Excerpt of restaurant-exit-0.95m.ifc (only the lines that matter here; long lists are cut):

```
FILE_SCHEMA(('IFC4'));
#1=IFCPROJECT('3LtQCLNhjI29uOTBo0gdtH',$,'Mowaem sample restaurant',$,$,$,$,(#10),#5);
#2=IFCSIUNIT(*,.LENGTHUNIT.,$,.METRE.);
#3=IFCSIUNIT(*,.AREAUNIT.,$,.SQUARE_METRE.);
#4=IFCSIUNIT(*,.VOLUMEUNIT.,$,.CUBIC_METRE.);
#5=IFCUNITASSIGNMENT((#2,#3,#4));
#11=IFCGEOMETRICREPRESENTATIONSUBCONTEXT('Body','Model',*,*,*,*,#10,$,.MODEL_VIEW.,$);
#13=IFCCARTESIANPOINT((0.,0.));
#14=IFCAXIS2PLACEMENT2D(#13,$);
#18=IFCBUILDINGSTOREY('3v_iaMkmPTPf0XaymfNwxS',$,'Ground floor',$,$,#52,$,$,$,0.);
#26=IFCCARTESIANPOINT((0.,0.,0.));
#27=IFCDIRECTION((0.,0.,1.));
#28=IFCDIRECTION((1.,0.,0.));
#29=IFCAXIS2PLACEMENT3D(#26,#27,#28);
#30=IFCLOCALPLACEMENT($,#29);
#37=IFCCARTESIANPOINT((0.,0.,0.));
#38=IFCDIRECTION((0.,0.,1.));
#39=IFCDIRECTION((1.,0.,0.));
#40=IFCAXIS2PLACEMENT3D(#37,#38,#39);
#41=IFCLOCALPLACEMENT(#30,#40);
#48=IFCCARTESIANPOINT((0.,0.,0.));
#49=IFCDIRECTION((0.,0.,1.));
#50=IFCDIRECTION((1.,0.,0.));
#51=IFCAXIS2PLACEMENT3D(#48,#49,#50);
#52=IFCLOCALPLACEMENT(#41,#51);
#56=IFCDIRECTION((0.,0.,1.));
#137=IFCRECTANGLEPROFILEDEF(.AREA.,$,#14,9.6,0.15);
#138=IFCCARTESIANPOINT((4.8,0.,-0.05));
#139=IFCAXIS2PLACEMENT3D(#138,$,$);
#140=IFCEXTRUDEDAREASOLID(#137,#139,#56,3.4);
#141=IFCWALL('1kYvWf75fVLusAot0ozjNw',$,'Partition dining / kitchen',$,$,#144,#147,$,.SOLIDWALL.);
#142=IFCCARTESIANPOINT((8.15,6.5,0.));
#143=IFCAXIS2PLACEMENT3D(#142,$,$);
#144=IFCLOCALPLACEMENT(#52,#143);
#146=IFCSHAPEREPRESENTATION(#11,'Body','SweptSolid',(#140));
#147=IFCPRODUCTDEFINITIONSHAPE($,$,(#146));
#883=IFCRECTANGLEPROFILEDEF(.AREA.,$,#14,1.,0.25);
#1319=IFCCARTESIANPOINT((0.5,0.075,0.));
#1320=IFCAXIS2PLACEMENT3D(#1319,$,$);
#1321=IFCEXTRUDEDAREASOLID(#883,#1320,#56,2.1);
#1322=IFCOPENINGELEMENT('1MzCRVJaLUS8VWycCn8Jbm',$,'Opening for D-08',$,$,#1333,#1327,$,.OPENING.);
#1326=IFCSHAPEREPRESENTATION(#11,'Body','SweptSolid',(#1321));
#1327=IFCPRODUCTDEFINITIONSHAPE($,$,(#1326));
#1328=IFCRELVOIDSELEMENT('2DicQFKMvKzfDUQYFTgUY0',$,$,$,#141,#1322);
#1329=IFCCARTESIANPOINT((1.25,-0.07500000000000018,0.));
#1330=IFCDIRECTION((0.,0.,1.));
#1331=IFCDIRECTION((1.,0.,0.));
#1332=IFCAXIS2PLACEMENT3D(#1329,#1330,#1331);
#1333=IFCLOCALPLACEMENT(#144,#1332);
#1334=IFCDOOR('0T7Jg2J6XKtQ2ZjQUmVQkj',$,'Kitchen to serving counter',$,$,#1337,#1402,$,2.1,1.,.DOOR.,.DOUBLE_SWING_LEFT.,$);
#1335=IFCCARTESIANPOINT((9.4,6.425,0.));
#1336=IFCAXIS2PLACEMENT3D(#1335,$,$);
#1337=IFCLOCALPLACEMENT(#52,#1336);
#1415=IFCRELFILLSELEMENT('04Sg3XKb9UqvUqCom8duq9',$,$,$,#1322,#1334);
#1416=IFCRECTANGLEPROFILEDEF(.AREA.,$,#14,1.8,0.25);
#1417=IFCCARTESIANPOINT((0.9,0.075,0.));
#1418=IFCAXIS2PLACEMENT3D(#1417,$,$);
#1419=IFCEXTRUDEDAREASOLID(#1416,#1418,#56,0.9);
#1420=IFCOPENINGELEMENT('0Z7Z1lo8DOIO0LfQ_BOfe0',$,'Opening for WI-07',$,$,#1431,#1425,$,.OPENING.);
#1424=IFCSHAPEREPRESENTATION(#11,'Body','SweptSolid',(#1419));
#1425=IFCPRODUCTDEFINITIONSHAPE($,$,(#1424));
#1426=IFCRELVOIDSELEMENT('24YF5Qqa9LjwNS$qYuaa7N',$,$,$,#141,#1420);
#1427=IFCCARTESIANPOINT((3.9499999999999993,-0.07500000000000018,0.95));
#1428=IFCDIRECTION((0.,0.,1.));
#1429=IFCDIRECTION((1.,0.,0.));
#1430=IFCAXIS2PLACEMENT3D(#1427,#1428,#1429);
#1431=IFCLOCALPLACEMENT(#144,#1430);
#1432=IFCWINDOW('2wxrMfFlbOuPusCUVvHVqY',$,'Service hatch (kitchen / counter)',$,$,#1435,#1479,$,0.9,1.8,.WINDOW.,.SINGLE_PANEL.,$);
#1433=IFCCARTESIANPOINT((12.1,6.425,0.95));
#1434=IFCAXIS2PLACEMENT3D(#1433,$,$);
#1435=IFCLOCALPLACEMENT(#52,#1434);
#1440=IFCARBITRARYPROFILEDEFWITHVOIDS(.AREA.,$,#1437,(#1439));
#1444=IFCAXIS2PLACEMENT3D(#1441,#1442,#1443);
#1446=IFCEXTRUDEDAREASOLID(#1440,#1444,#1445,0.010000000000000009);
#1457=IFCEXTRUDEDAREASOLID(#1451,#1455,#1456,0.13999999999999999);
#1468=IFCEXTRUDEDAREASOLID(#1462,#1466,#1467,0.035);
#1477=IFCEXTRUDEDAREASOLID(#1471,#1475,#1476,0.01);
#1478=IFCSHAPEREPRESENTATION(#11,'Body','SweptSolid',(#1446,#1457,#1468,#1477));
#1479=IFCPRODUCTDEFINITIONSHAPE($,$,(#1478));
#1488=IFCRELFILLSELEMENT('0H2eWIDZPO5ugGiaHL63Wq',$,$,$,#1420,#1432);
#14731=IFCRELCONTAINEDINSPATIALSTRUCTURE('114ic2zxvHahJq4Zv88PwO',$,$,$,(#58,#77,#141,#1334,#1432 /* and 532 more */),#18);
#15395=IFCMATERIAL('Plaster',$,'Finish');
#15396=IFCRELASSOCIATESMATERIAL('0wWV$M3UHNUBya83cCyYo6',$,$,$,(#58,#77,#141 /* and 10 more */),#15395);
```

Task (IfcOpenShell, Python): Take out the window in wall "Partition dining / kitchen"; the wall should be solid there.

```python
import ifcopenshell
import ifcopenshell.api.feature
import ifcopenshell.api.root
import ifcopenshell.geom
import ifcopenshell.util.shape

model = ifcopenshell.open("restaurant-exit-0.95m.ifc")
settings = ifcopenshell.geom.settings()


def volume(element):
    """Net volume in cubic metres, openings subtracted."""
    shape = ifcopenshell.geom.create_shape(settings, element)
    return ifcopenshell.util.shape.get_volume(shape.geometry)


window = model.by_guid("2wxrMfFlbOuPusCUVvHVqY")
opening = window.FillsVoids[0].RelatingOpeningElement
wall = opening.VoidsElements[0].RelatingBuildingElement
before = volume(wall)

ifcopenshell.api.root.remove_product(model, product=window)
ifcopenshell.api.feature.remove_feature(model, feature=opening)

after = volume(wall)

print(f"wall volume {before:.3f} -> {after:.3f} m3")

model.write("restaurant-exit-0.95m_v2.ifc")
```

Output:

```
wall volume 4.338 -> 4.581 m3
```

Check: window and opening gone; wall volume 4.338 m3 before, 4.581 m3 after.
